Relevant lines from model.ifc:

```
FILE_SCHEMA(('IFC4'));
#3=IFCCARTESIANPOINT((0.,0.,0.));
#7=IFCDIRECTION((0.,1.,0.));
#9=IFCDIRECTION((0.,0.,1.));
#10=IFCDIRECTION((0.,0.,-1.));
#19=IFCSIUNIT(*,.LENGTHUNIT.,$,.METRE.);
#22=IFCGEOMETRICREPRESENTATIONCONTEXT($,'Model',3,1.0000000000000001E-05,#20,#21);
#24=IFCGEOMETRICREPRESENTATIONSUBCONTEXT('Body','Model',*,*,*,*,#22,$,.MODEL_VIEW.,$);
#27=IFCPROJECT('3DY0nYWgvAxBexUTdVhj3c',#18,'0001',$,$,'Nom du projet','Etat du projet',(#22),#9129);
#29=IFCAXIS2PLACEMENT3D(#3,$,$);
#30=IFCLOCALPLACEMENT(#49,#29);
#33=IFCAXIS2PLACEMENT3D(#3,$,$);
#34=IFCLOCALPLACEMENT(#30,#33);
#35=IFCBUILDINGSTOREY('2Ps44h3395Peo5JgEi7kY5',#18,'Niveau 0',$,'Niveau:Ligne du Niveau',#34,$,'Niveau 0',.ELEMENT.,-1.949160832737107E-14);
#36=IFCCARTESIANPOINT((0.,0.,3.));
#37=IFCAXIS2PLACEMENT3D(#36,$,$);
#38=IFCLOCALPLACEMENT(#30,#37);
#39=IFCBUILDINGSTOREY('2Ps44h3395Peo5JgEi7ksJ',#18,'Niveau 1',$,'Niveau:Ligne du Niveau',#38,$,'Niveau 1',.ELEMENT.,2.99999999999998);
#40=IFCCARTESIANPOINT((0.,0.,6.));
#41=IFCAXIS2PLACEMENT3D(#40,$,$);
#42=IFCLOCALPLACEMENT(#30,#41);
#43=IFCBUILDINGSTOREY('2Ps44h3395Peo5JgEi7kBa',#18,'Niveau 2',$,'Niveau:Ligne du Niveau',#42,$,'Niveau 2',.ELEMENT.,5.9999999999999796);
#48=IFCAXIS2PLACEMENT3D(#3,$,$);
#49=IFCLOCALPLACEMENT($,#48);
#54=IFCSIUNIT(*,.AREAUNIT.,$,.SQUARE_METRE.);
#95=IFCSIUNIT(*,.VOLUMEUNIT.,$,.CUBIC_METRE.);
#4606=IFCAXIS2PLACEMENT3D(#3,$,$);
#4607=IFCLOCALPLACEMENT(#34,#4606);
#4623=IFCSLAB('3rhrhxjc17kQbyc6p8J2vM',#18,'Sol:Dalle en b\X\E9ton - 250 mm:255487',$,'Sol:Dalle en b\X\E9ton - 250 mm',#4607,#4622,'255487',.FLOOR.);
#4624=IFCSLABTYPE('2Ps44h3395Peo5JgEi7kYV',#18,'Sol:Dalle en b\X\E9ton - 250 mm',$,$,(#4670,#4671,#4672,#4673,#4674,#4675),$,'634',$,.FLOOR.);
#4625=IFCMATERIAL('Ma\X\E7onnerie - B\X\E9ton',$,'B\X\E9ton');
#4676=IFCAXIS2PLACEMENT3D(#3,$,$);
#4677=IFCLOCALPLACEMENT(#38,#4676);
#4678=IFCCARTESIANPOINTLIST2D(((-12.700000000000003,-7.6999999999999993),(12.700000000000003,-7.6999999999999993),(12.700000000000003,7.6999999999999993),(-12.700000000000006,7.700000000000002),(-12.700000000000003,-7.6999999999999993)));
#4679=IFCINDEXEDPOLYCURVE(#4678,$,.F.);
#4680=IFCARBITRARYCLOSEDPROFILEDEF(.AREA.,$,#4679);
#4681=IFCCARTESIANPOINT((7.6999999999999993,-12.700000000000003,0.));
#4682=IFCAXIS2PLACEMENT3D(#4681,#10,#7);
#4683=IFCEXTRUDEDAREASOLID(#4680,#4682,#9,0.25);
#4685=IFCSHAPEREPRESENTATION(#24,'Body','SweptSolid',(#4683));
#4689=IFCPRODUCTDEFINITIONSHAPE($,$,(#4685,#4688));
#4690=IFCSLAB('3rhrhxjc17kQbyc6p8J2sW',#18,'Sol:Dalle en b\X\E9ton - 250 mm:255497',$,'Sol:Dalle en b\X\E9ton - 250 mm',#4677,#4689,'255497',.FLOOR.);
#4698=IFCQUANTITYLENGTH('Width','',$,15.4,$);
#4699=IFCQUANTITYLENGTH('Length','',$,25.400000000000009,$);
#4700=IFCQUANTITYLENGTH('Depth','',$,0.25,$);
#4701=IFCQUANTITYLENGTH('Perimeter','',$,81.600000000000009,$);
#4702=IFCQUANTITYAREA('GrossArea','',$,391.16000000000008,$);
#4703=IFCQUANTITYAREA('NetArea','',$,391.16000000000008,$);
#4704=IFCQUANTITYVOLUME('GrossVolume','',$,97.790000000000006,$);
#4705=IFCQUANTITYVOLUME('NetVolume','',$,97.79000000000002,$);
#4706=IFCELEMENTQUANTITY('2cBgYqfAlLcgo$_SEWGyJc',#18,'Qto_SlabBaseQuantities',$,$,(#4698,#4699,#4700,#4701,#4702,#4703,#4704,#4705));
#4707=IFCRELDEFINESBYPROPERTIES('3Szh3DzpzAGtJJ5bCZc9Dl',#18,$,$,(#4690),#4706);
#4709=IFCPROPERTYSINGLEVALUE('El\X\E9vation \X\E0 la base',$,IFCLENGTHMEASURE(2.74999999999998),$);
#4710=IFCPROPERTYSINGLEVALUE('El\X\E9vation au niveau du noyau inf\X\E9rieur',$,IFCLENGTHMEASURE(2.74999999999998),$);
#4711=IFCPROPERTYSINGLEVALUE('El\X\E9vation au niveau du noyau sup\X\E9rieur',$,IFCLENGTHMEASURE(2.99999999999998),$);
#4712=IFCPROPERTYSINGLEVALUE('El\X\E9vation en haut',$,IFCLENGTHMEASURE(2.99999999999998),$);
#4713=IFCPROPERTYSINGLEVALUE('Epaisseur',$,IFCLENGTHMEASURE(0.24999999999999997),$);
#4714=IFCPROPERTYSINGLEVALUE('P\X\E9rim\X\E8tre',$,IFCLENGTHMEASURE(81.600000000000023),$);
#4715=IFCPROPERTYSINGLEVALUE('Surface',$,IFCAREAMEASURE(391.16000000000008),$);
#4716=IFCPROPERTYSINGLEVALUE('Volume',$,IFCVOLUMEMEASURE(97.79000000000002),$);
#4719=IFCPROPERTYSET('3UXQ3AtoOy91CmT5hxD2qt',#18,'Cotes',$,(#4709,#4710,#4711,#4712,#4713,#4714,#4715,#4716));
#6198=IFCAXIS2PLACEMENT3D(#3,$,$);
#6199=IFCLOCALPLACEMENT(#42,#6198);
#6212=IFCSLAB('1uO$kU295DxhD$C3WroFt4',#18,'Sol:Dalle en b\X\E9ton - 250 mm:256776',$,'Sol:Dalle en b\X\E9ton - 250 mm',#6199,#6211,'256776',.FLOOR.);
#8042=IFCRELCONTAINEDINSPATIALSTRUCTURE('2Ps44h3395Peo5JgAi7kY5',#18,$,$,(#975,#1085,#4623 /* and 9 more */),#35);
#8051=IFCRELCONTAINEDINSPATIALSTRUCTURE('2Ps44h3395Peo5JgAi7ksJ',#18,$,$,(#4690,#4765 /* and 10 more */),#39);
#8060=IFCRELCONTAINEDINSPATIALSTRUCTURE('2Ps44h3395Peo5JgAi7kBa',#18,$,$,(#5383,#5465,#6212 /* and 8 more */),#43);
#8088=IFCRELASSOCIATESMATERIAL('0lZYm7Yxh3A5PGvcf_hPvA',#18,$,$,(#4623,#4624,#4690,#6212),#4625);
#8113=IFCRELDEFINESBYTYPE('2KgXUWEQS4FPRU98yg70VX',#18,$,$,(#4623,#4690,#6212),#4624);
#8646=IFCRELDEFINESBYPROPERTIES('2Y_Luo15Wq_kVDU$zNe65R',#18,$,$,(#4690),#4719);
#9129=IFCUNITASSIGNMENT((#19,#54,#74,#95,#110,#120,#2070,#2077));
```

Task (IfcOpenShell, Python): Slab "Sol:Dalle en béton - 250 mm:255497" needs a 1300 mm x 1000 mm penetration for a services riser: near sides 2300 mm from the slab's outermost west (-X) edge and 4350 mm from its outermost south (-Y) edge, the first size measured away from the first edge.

```python
import numpy as np
import ifcopenshell
import ifcopenshell.api.feature
import ifcopenshell.api.geometry
import ifcopenshell.api.pset
import ifcopenshell.api.root
import ifcopenshell.geom
import ifcopenshell.util.element
import ifcopenshell.util.placement
import ifcopenshell.util.representation
import ifcopenshell.util.shape
import ifcopenshell.util.unit

model = ifcopenshell.open("model.ifc")
unit_scale = ifcopenshell.util.unit.calculate_unit_scale(model)
area_scale = ifcopenshell.util.unit.calculate_unit_scale(model, "AREAUNIT")
volume_scale = ifcopenshell.util.unit.calculate_unit_scale(model, "VOLUMEUNIT")
settings = ifcopenshell.geom.settings()


def volume(element):
    """Net volume in cubic metres, openings subtracted."""
    shape = ifcopenshell.geom.create_shape(settings, element)
    return ifcopenshell.util.shape.get_volume(shape.geometry)


slab = model.by_guid("3rhrhxjc17kQbyc6p8J2sW")
before = volume(slab)

# Extent in the slab's own axes, in metres. The edges named are its -X and -Y sides.
slab_shape = ifcopenshell.geom.create_shape(settings, slab)
vertices = ifcopenshell.util.shape.get_vertices(slab_shape.geometry)
x_min, y_min, bottom = vertices.min(axis=0)
top = vertices[:, 2].max()

opening = ifcopenshell.api.root.create_entity(model, ifc_class="IfcOpeningElement", name="Services riser opening", predefined_type="OPENING")
context = ifcopenshell.util.representation.get_context(model, "Model", "Body", "MODEL_VIEW")
width, depth = 1.3, 1
outline = [(0.0, 0.0), (width, 0.0), (width, depth), (0.0, depth), (0.0, 0.0)]
# Overshoot both faces by 50 mm so the cut is clean.
shape = ifcopenshell.api.geometry.add_slab_representation(
    model, context=context, depth=top - bottom + 0.1, polyline=outline
)
ifcopenshell.api.geometry.assign_representation(model, product=opening, representation=shape)

matrix = ifcopenshell.util.placement.get_local_placement(slab.ObjectPlacement)
matrix[:, 3] = matrix @ np.append(np.array([x_min + 2.3, y_min + 4.35, bottom - 0.05]) / unit_scale, 1.0)
ifcopenshell.api.geometry.edit_object_placement(model, product=opening, matrix=matrix, is_si=False)
ifcopenshell.api.feature.add_feature(model, feature=opening, element=slab)

after = volume(slab)

# Update the slab's stored quantities.
qto = model.by_id(ifcopenshell.util.element.get_pset(slab, "Qto_SlabBaseQuantities", should_inherit=False)["id"])
ifcopenshell.api.pset.edit_qto(model, qto=qto, properties={
    "NetArea": after / (top - bottom) / area_scale,
    "NetVolume": after / volume_scale,
})
pset = model.by_id(ifcopenshell.util.element.get_pset(slab, "Cotes", should_inherit=False)["id"])
ifcopenshell.api.pset.edit_pset(model, pset=pset, properties={
    "Surface": model.create_entity("IfcAreaMeasure", after / (top - bottom) / area_scale),
    "Volume": model.create_entity("IfcVolumeMeasure", after / volume_scale),
})

print(f"slab volume {before:.3f} -> {after:.3f} m3")

model.write("model_edited.ifc")
```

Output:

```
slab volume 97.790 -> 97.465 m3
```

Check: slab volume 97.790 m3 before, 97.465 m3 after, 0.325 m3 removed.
